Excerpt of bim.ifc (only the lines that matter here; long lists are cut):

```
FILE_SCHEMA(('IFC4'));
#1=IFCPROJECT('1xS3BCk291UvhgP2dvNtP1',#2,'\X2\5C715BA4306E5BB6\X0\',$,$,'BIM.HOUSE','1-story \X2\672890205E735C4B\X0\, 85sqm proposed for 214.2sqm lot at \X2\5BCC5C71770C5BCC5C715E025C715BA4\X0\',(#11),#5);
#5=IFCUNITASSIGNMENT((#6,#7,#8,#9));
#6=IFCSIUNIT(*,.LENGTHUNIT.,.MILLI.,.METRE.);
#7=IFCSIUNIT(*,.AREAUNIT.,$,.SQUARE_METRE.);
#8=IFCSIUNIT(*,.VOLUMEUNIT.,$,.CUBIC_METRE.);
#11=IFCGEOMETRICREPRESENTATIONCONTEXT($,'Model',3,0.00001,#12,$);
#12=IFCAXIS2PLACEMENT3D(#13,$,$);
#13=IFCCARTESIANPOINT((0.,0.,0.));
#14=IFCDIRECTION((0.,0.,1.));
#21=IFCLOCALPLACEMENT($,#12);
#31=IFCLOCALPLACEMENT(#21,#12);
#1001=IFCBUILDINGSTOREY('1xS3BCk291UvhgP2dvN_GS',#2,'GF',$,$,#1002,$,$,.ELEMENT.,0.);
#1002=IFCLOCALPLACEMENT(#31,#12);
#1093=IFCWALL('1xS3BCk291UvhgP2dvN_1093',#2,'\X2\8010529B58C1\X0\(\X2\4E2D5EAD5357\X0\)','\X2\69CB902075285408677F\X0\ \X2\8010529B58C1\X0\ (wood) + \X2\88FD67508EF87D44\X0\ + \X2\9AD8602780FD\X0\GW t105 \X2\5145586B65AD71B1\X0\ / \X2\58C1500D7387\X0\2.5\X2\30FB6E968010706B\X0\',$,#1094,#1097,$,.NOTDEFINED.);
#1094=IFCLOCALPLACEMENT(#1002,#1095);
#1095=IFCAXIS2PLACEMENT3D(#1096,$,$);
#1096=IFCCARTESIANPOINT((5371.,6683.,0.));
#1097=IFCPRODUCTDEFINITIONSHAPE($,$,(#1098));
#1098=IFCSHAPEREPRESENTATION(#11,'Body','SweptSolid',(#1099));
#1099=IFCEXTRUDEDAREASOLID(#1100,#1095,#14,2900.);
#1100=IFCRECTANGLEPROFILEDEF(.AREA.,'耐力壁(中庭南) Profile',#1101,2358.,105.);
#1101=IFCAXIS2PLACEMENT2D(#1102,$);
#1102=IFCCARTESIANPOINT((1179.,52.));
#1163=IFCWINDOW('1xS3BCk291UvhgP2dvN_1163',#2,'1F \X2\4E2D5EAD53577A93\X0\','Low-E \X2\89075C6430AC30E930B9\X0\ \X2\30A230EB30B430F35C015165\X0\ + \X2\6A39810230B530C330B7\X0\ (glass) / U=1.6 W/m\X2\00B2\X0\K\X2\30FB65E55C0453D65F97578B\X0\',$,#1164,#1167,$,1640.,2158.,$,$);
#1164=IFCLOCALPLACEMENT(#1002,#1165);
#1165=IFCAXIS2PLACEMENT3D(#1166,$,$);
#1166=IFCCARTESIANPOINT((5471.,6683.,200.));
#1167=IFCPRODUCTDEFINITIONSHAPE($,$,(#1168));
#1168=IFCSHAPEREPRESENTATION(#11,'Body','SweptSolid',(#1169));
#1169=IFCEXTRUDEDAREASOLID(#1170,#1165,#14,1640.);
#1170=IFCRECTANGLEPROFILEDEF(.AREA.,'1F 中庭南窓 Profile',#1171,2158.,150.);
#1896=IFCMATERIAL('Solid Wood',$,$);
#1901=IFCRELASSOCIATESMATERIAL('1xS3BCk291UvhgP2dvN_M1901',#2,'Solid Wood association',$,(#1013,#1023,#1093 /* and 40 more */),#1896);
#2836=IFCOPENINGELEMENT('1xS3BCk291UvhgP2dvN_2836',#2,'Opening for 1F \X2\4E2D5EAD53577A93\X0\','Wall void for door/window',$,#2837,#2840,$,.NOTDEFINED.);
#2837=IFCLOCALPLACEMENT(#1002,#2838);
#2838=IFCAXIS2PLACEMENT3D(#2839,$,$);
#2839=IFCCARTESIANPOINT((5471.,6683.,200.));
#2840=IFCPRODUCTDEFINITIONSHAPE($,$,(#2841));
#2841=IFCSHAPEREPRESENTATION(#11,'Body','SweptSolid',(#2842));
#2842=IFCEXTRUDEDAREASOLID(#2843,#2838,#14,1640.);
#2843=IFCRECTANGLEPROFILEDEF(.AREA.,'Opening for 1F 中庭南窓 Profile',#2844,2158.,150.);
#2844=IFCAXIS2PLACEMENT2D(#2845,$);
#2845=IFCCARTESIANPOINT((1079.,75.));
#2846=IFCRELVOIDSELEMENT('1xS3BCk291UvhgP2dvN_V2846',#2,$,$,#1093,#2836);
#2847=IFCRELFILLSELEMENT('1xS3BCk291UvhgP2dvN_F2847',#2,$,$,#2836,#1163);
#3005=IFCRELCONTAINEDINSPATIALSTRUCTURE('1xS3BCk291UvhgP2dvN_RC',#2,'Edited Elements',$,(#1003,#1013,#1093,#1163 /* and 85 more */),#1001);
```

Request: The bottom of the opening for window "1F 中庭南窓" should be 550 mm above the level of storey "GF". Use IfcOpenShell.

```python
import numpy as np
import ifcopenshell
import ifcopenshell.api.geometry
import ifcopenshell.geom
import ifcopenshell.util.element
import ifcopenshell.util.placement
import ifcopenshell.util.shape
import ifcopenshell.util.unit

model = ifcopenshell.open("bim.ifc")
unit_scale = ifcopenshell.util.unit.calculate_unit_scale(model)

window = model.by_id(1163)
opening = window.FillsVoids[0].RelatingOpeningElement
storey = ifcopenshell.util.element.get_container(window, ifc_class="IfcBuildingStorey")
level = ifcopenshell.util.placement.get_local_placement(storey.ObjectPlacement)[2, 3]

# The opening's origin need not be at the sill, so measure its lowest point.
shape = ifcopenshell.geom.create_shape(ifcopenshell.geom.settings(), opening)
bottom = ifcopenshell.util.shape.get_shape_bottom_elevation(shape, shape.geometry) / unit_scale
dz = level + 0.55 / unit_scale - bottom

shift = np.array([0.0, 0.0, dz])
# The window is not placed relative to its opening, so move both.
for product in (opening, window):
    matrix = ifcopenshell.util.placement.get_local_placement(product.ObjectPlacement)
    matrix[:3, 3] += shift
    ifcopenshell.api.geometry.edit_object_placement(model, product=product, matrix=matrix, is_si=False)

print(f"moved by {dz * unit_scale:+.3f} m")

model.write("bim-out.ifc")
```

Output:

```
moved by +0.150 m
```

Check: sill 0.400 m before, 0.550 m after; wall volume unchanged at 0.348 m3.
